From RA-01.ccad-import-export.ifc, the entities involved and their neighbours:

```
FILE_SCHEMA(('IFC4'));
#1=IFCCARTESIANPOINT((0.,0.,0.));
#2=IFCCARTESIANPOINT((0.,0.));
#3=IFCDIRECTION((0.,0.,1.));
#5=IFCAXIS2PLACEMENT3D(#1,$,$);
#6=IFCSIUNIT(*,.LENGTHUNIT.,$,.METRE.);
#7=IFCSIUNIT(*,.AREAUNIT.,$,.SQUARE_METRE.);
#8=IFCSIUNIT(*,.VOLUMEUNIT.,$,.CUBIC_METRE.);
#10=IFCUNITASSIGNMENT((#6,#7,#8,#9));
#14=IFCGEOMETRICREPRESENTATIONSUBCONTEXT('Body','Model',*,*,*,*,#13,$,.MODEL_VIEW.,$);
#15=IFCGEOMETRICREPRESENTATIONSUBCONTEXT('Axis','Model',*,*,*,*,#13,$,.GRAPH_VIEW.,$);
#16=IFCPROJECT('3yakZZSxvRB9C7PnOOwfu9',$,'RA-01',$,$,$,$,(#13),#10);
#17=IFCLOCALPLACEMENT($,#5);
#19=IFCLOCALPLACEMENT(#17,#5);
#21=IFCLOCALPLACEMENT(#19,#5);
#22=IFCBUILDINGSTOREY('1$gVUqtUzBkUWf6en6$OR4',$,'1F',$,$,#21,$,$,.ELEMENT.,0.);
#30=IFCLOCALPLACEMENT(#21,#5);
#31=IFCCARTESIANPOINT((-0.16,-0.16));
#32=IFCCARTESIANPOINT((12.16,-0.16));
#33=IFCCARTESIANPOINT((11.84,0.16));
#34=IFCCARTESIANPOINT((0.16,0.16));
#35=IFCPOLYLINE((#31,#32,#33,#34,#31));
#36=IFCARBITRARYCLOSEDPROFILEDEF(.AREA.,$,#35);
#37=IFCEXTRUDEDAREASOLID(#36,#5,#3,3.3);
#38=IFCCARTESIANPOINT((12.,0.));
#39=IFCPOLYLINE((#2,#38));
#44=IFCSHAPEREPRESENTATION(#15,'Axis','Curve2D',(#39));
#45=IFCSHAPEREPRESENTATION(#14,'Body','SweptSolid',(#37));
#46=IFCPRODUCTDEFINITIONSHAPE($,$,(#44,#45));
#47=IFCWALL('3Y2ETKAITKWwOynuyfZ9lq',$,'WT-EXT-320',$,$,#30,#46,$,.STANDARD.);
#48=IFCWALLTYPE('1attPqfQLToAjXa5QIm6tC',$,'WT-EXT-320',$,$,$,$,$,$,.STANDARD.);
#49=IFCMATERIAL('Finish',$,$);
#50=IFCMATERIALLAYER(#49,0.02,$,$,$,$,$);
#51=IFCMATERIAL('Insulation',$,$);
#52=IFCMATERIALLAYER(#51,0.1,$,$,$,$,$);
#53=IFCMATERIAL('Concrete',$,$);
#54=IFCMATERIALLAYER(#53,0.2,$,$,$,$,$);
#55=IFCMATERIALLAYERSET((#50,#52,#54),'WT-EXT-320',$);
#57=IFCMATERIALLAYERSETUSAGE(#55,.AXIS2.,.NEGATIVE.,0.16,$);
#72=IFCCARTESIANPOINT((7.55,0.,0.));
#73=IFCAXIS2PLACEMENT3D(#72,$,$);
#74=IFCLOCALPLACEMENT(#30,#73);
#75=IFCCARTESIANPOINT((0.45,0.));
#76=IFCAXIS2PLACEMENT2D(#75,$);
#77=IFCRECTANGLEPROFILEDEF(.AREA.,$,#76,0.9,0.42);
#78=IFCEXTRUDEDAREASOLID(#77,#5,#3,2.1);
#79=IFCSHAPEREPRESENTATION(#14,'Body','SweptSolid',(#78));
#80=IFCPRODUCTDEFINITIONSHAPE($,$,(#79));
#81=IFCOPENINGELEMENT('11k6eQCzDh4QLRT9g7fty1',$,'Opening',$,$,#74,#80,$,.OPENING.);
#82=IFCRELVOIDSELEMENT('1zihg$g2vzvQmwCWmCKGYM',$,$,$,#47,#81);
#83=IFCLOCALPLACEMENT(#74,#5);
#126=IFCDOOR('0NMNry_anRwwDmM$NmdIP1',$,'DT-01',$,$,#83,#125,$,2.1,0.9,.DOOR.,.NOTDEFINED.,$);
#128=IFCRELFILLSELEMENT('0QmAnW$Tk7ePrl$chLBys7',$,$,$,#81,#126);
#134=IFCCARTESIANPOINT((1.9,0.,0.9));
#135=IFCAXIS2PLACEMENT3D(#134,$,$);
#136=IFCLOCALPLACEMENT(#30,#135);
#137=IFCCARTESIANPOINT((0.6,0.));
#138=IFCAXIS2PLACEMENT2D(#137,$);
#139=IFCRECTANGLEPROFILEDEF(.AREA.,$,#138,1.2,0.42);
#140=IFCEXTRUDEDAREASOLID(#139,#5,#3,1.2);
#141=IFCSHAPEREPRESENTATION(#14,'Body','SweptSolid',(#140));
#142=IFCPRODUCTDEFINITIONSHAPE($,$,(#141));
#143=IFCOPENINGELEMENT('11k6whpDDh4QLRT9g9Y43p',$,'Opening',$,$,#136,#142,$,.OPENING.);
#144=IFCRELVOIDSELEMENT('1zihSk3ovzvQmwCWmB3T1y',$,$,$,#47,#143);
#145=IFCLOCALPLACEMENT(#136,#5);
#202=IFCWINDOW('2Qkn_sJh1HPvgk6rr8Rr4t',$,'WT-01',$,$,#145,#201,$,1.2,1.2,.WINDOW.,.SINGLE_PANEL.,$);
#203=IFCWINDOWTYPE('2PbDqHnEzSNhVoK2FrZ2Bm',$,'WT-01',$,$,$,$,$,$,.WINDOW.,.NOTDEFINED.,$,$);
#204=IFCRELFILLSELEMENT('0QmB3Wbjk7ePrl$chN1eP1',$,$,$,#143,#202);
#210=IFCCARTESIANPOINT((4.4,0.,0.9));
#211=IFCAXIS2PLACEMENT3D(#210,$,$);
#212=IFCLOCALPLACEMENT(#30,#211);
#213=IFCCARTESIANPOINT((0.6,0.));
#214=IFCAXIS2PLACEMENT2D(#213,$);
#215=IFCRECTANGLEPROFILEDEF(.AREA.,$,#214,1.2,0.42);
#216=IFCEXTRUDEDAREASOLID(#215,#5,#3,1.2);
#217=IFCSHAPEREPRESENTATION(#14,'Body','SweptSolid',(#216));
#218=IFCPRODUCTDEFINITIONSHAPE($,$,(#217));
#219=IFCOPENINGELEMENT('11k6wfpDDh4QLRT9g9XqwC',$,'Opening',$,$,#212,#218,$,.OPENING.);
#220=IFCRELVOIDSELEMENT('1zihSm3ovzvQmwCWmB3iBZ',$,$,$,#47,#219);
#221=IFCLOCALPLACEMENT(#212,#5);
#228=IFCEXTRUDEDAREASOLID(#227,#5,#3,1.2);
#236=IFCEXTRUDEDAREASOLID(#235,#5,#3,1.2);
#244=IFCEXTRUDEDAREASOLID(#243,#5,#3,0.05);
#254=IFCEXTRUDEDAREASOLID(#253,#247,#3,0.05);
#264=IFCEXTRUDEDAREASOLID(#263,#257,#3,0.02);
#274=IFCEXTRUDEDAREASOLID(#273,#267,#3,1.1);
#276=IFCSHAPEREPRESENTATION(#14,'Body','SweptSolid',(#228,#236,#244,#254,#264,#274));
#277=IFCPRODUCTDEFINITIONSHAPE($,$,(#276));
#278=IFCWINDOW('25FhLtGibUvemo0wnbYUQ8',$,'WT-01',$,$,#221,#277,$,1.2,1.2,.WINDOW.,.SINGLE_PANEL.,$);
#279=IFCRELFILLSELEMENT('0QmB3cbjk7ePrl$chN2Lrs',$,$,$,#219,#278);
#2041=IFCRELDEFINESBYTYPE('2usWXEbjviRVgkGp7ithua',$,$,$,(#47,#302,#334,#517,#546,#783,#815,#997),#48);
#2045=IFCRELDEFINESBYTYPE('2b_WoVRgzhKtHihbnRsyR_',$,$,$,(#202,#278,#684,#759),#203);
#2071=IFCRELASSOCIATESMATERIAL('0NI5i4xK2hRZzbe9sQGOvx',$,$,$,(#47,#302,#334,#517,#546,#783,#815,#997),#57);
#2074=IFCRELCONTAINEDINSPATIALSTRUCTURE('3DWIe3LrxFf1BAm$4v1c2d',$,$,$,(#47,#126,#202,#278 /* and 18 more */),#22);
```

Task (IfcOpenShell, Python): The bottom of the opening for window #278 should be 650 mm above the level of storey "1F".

```python
import numpy as np
import ifcopenshell
import ifcopenshell.api.geometry
import ifcopenshell.geom
import ifcopenshell.util.element
import ifcopenshell.util.placement
import ifcopenshell.util.shape
import ifcopenshell.util.unit

model = ifcopenshell.open("RA-01.ccad-import-export.ifc")
unit_scale = ifcopenshell.util.unit.calculate_unit_scale(model)

window = model.by_id(278)
opening = window.FillsVoids[0].RelatingOpeningElement
storey = ifcopenshell.util.element.get_container(window, ifc_class="IfcBuildingStorey")
level = ifcopenshell.util.placement.get_local_placement(storey.ObjectPlacement)[2, 3]

# The opening's origin need not be at the sill, so measure its lowest point.
shape = ifcopenshell.geom.create_shape(ifcopenshell.geom.settings(), opening)
bottom = ifcopenshell.util.shape.get_shape_bottom_elevation(shape, shape.geometry) / unit_scale
dz = level + 0.65 / unit_scale - bottom

shift = np.array([0.0, 0.0, dz])
# The window is placed relative to its opening, so it follows when the opening moves.
matrix = ifcopenshell.util.placement.get_local_placement(opening.ObjectPlacement)
matrix[:3, 3] += shift
ifcopenshell.api.geometry.edit_object_placement(
    model, product=opening, matrix=matrix, is_si=False, should_transform_children=True
)

print(f"moved by {dz * unit_scale:+.3f} m")

model.write("RA-01.ccad-import-export_updated.ifc")
```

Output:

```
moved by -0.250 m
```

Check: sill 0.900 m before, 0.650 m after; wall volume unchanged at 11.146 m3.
